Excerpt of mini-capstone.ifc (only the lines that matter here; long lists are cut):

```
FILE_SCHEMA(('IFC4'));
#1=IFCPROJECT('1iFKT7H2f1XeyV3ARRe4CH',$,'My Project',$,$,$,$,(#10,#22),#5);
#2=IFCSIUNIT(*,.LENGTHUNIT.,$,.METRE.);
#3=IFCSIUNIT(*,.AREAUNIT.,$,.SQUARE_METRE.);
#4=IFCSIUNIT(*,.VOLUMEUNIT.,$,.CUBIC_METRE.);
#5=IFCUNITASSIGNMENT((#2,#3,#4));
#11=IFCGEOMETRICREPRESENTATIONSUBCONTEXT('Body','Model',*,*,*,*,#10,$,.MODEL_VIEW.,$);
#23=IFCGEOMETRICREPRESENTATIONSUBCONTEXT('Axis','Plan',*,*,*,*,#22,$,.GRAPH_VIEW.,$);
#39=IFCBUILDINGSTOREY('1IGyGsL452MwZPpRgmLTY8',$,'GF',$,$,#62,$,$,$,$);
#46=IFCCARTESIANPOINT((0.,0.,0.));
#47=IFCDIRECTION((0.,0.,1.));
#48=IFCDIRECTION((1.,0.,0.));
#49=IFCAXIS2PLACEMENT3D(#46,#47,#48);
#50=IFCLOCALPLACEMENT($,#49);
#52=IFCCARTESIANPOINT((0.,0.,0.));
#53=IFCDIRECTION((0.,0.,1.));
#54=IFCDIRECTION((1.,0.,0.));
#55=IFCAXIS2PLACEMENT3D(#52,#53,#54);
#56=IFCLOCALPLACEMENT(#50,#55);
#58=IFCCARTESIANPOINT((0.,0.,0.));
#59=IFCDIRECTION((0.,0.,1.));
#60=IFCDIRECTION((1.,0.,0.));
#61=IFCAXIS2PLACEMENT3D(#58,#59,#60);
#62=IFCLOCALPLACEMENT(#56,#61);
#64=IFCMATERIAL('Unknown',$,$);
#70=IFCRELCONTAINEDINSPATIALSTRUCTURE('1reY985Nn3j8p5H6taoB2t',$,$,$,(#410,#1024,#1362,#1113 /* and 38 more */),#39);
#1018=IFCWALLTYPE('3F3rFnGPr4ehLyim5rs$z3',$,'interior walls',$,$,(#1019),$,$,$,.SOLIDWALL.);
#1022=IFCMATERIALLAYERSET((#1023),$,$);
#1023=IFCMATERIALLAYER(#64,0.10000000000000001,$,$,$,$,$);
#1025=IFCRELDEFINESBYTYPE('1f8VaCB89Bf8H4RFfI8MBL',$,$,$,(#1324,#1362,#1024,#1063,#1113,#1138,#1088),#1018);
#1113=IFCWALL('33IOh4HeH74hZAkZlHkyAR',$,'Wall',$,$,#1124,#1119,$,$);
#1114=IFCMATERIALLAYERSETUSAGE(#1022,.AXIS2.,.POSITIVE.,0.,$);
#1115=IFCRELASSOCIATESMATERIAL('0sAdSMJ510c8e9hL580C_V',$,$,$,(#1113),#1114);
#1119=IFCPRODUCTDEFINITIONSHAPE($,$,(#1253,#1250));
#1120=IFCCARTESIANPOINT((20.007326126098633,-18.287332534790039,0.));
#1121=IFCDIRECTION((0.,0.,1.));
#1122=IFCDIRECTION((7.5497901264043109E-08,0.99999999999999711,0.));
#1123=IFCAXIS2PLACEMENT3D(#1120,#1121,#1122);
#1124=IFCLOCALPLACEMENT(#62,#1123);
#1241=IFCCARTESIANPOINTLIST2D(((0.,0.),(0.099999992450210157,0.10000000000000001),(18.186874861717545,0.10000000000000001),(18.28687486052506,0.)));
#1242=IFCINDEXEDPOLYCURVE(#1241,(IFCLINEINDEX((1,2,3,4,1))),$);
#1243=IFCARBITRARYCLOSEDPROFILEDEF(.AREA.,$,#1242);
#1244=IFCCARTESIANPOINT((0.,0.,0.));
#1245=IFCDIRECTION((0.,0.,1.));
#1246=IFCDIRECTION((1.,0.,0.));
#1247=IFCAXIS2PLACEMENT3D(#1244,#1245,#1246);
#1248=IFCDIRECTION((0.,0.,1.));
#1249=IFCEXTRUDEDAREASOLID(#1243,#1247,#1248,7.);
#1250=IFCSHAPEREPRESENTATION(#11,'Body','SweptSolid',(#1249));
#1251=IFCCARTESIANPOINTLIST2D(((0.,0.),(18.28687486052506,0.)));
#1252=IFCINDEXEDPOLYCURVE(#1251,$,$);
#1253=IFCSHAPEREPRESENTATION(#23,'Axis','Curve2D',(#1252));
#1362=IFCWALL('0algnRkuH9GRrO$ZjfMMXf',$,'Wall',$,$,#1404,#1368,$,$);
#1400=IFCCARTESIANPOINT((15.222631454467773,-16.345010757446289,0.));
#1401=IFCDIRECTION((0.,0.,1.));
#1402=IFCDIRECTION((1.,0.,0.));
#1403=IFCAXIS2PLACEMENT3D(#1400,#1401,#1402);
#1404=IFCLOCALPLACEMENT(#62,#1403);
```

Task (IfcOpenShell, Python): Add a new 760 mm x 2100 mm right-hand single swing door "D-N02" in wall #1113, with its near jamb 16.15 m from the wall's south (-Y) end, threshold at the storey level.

```python
import numpy as np
import ifcopenshell
import ifcopenshell.api.feature
import ifcopenshell.api.geometry
import ifcopenshell.api.root
import ifcopenshell.api.spatial
import ifcopenshell.geom
import ifcopenshell.util.element
import ifcopenshell.util.placement
import ifcopenshell.util.representation
import ifcopenshell.util.shape
import ifcopenshell.util.unit

model = ifcopenshell.open("mini-capstone.ifc")
unit_scale = ifcopenshell.util.unit.calculate_unit_scale(model)
settings = ifcopenshell.geom.settings()


def volume(element):
    """Net volume in cubic metres, openings subtracted."""
    shape = ifcopenshell.geom.create_shape(settings, element)
    return ifcopenshell.util.shape.get_volume(shape.geometry)


wall = model.by_guid("33IOh4HeH74hZAkZlHkyAR")
storey = ifcopenshell.util.element.get_container(wall, ifc_class="IfcBuildingStorey")
context = ifcopenshell.util.representation.get_context(model, "Model", "Body", "MODEL_VIEW")
before = volume(wall)

width, height, from_end, sill = 0.76, 2.1, 16.15, 0.0  # metres

# The wall runs along its own X axis, and the end named is its -X end.
wall_shape = ifcopenshell.geom.create_shape(settings, wall)
x, y, z = ifcopenshell.util.shape.get_vertices(wall_shape.geometry).T
start = x.min() + from_end
face, thickness = float(y.min()), float(y.max() - y.min())
wall_matrix = ifcopenshell.util.placement.get_local_placement(wall.ObjectPlacement)
level = ifcopenshell.util.placement.get_local_placement(storey.ObjectPlacement)[2, 3]


def in_wall(x, y):
    """Placement at x, y metres in the wall's axes, at sill height."""
    matrix = wall_matrix.copy()
    matrix[:, 3] = wall_matrix @ np.array([x / unit_scale, y / unit_scale, 0.0, 1.0])
    matrix[2, 3] = level + sill / unit_scale
    return matrix


# Opening: a box that overshoots both wall faces by 50 mm.
opening = ifcopenshell.api.root.create_entity(model, ifc_class="IfcOpeningElement", predefined_type="OPENING")
box = ifcopenshell.api.geometry.add_wall_representation(
    model, context=context, length=width, height=height, thickness=thickness + 0.1
)
ifcopenshell.api.geometry.assign_representation(model, product=opening, representation=box)
ifcopenshell.api.geometry.edit_object_placement(model, product=opening, matrix=in_wall(start, face - 0.05), is_si=False)
ifcopenshell.api.feature.add_feature(model, feature=opening, element=wall)

door = ifcopenshell.api.root.create_entity(model, ifc_class="IfcDoor", name="D-N02", predefined_type="DOOR")
door.OverallWidth, door.OverallHeight = width / unit_scale, height / unit_scale
door.OperationType = "SINGLE_SWING_RIGHT"
body = ifcopenshell.api.geometry.add_door_representation(
    model,
    context=context,
    overall_width=door.OverallWidth,
    overall_height=door.OverallHeight,
    operation_type="SINGLE_SWING_RIGHT",
    lining_properties={"LiningDepth": thickness / unit_scale, "ThresholdDepth": thickness / unit_scale},
)
ifcopenshell.api.geometry.assign_representation(model, product=door, representation=body)
ifcopenshell.api.spatial.assign_container(model, products=[door], relating_structure=storey)
ifcopenshell.api.feature.add_filling(model, opening=opening, element=door)

# The lining spans the wall, so the door starts at the wall face.
ifcopenshell.api.geometry.edit_object_placement(model, product=door, matrix=in_wall(start, face), is_si=False)

after = volume(wall)

print(f"wall volume {before:.3f} -> {after:.3f} m3")

model.write("mini-capstone_rev.ifc")
```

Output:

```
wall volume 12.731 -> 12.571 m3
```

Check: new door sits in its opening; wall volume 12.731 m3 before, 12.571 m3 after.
